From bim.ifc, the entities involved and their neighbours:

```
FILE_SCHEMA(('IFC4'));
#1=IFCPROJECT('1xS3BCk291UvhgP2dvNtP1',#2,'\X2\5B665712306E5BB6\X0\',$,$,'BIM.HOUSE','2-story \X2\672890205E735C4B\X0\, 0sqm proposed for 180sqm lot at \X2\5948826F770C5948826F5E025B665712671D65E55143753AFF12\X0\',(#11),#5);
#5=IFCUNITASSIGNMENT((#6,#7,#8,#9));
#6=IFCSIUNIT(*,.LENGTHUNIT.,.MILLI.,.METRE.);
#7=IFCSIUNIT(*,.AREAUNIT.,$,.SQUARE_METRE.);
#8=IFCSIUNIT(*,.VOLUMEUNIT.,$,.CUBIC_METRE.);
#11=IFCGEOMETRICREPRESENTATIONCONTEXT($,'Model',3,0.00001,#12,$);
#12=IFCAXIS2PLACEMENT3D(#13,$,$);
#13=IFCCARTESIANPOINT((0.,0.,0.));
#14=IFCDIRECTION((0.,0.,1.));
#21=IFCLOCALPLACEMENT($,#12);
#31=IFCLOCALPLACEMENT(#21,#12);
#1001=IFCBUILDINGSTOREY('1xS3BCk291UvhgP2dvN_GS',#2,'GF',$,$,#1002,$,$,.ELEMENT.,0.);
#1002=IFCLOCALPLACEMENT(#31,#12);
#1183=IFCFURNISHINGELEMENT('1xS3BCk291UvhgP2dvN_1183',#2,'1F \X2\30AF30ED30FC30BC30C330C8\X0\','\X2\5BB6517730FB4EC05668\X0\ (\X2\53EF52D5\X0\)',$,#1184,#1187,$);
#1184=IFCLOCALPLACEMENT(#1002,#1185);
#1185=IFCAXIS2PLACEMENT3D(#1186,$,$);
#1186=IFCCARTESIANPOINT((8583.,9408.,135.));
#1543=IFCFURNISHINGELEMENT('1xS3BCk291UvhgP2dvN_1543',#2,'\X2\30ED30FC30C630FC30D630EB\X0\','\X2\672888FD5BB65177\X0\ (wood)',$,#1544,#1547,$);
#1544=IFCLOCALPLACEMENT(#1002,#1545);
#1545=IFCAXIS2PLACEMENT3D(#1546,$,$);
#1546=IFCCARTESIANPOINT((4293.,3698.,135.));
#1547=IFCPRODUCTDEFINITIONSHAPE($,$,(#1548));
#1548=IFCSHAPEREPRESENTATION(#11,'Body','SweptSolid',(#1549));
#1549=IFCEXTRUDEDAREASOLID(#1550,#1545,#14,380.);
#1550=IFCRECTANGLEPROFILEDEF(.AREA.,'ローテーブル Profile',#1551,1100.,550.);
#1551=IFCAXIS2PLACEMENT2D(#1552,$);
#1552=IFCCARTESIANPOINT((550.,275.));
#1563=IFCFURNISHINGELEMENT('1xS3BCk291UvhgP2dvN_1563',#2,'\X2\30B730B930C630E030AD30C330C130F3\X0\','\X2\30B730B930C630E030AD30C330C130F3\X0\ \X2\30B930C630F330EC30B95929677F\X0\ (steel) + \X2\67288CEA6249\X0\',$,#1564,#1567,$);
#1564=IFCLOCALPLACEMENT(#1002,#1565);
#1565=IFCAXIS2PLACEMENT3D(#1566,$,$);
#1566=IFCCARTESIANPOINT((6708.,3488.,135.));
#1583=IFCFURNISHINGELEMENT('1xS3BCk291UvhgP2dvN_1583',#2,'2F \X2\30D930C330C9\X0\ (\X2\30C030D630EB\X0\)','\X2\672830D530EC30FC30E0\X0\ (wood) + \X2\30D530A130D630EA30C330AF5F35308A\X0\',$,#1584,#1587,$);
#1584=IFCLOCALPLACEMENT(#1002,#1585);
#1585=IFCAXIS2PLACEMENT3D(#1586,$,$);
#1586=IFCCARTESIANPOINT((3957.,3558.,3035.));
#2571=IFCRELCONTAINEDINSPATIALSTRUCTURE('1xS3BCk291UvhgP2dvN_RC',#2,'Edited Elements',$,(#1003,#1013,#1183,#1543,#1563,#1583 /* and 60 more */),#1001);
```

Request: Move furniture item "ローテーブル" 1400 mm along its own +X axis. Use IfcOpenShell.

```python
import ifcopenshell
import ifcopenshell.api.geometry
import ifcopenshell.util.placement
import ifcopenshell.util.unit

model = ifcopenshell.open("bim.ifc")
unit_scale = ifcopenshell.util.unit.calculate_unit_scale(model)

item = model.by_guid("1xS3BCk291UvhgP2dvN_1543")
matrix = ifcopenshell.util.placement.get_local_placement(item.ObjectPlacement)
matrix[:3, 3] += matrix[:3, 0] * 1.4 / unit_scale
ifcopenshell.api.geometry.edit_object_placement(model, product=item, matrix=matrix, is_si=False)

print(ifcopenshell.util.placement.get_local_placement(item.ObjectPlacement).round(3) + 0.0)

model.write("bim_updated.ifc")
```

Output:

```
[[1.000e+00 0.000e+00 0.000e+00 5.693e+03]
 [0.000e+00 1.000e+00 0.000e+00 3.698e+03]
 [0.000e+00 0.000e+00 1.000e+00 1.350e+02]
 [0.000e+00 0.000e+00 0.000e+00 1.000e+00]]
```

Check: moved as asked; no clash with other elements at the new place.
